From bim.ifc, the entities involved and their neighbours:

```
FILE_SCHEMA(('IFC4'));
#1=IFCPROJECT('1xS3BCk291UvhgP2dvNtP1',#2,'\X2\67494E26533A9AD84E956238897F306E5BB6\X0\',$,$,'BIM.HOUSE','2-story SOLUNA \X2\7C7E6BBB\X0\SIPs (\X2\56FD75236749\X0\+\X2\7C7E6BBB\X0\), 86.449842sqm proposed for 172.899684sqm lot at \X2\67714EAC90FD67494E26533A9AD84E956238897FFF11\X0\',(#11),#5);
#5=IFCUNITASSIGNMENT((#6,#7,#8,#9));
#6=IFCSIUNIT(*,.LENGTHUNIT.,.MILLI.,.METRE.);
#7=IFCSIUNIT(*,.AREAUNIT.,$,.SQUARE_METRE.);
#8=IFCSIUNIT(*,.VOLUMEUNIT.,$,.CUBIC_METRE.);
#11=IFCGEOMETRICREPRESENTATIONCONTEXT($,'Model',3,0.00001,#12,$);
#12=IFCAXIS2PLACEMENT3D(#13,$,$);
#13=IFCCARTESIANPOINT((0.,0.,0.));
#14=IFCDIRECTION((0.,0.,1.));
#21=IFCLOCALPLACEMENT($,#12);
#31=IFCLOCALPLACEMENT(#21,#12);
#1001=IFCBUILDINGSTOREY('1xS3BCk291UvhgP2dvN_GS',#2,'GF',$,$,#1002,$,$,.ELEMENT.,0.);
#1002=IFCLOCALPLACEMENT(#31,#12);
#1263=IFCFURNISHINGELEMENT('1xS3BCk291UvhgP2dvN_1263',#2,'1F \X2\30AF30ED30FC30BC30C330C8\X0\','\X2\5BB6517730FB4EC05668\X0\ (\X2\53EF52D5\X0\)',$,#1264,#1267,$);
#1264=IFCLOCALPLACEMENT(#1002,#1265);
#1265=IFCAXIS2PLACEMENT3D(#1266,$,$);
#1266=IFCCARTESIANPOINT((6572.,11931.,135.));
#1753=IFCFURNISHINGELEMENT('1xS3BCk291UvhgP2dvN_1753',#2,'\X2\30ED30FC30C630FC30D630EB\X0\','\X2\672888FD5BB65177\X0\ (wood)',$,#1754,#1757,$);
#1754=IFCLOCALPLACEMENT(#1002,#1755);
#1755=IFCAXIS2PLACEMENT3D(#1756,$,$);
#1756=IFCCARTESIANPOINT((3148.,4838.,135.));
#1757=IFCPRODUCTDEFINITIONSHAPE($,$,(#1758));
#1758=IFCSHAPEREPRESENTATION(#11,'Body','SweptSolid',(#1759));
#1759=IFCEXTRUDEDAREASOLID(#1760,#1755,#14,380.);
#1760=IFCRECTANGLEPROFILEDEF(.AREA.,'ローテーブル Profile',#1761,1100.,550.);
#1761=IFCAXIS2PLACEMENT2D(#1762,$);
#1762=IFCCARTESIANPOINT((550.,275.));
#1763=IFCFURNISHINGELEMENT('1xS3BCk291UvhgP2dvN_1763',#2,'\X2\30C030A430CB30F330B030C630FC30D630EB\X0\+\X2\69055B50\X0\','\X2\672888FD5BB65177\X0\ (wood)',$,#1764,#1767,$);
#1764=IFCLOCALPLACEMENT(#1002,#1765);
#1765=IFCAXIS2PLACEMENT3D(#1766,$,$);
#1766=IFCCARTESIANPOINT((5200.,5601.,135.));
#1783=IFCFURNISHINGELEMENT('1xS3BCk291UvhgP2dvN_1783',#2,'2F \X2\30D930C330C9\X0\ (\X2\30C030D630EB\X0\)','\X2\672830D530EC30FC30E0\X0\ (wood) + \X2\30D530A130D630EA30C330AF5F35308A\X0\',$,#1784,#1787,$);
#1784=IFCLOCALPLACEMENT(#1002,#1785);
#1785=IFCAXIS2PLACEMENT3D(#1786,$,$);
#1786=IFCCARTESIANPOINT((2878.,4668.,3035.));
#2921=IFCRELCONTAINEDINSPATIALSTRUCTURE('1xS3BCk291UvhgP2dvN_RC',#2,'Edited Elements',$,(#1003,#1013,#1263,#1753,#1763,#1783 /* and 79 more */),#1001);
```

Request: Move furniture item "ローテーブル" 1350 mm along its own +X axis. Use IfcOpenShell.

```python
import ifcopenshell
import ifcopenshell.api.geometry
import ifcopenshell.util.placement

model = ifcopenshell.open("bim.ifc")

item = model.by_guid("1xS3BCk291UvhgP2dvN_1753")
matrix = ifcopenshell.util.placement.get_local_placement(item.ObjectPlacement)
matrix[:3, 3] += matrix[:3, 0] * 1350.0
ifcopenshell.api.geometry.edit_object_placement(model, product=item, matrix=matrix, is_si=False)

print(ifcopenshell.util.placement.get_local_placement(item.ObjectPlacement).round(3) + 0.0)

model.write("bim_rev.ifc")
```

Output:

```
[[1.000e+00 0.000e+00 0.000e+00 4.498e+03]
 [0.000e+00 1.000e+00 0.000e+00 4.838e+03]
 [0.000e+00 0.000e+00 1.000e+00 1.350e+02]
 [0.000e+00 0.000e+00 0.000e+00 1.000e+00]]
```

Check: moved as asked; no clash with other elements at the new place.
